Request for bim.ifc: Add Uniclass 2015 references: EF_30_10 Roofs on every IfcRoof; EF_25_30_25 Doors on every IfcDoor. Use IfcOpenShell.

First a look at what the model holds.

```python
import ifcopenshell

model = ifcopenshell.open("bim.ifc")
print(model.schema)
print("classifications:", [c.Name for c in model.by_type("IfcClassification")])
for ifc_class in ("IfcDoor", "IfcRoof", "IfcStair", "IfcWall", "IfcWindow"):
    print(ifc_class, len(model.by_type(ifc_class)))
```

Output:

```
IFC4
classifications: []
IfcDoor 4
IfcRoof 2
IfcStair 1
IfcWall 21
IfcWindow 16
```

```python
import ifcopenshell
import ifcopenshell.api.classification

model = ifcopenshell.open("bim.ifc")

system = ifcopenshell.api.classification.add_classification(model, classification="Uniclass 2015")

codes = {
    "IfcRoof": ("EF_30_10", "Roofs"),
    "IfcDoor": ("EF_25_30_25", "Doors"),
}
for ifc_class, (code, name) in codes.items():
    products = model.by_type(ifc_class)
    ifcopenshell.api.classification.add_reference(
        model, products=products, classification=system, identification=code, name=name
    )
    print(code, len(products))

model.write("bim-out.ifc")
```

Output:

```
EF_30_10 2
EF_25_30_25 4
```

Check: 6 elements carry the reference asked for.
